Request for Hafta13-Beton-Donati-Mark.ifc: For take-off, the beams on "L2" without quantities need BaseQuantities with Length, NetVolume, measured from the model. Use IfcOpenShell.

First a look at what the model holds.

```python
import ifcopenshell
import ifcopenshell.util.element
import ifcopenshell.util.unit

model = ifcopenshell.open("Hafta13-Beton-Donati-Mark.ifc")
print(model.schema)
for unit_type in ("LENGTHUNIT", "AREAUNIT", "VOLUMEUNIT"):
    print(unit_type, ifcopenshell.util.unit.calculate_unit_scale(model, unit_type))
storey = next(s for s in model.by_type("IfcBuildingStorey") if s.Name == "L2")
beams = [e for e in ifcopenshell.util.element.get_decomposition(storey) if e.is_a("IfcBeam")]
for e in sorted(beams, key=lambda e: e.id()):
    print(e.id(), e.is_a(), e.Name, list(ifcopenshell.util.element.get_psets(e, qtos_only=True)), sep=" | ")
```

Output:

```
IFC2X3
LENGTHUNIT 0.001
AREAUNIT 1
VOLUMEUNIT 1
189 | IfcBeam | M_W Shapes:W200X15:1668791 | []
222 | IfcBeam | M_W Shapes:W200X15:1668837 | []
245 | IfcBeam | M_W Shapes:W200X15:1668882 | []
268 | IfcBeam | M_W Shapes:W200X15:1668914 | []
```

```python
import ifcopenshell
import ifcopenshell.api.pset
import ifcopenshell.geom
import ifcopenshell.util.element
import ifcopenshell.util.shape
import ifcopenshell.util.unit

model = ifcopenshell.open("Hafta13-Beton-Donati-Mark.ifc")
unit_scale = ifcopenshell.util.unit.calculate_unit_scale(model)
volume_scale = ifcopenshell.util.unit.calculate_unit_scale(model, "VOLUMEUNIT")
settings = ifcopenshell.geom.settings()

storey = next(s for s in model.by_type("IfcBuildingStorey") if s.Name == "L2")
beams = [e for e in ifcopenshell.util.element.get_decomposition(storey) if e.is_a("IfcBeam")]

for e in sorted(beams, key=lambda e: e.id()):
    if ifcopenshell.util.element.get_psets(e, qtos_only=True, should_inherit=False):
        continue
    # Geometry comes back in metres, in the element's own axes.
    shape = ifcopenshell.geom.create_shape(settings, e)
    values = {
        "Length": ifcopenshell.util.shape.get_max_xyz(shape.geometry) / unit_scale,
        "NetVolume": ifcopenshell.util.shape.get_volume(shape.geometry) / volume_scale,
    }
    qto = ifcopenshell.api.pset.add_qto(model, product=e, name="BaseQuantities")
    ifcopenshell.api.pset.edit_qto(model, qto=qto, properties=values)
    print(e.id(), {k: round(v, 3) for k, v in values.items()})

model.write("Hafta13-Beton-Donati-Mark_updated.ifc")
```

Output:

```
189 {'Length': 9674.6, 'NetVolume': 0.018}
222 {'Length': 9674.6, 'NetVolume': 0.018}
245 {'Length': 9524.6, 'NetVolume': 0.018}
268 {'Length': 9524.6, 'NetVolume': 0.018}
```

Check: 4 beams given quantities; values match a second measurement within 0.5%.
